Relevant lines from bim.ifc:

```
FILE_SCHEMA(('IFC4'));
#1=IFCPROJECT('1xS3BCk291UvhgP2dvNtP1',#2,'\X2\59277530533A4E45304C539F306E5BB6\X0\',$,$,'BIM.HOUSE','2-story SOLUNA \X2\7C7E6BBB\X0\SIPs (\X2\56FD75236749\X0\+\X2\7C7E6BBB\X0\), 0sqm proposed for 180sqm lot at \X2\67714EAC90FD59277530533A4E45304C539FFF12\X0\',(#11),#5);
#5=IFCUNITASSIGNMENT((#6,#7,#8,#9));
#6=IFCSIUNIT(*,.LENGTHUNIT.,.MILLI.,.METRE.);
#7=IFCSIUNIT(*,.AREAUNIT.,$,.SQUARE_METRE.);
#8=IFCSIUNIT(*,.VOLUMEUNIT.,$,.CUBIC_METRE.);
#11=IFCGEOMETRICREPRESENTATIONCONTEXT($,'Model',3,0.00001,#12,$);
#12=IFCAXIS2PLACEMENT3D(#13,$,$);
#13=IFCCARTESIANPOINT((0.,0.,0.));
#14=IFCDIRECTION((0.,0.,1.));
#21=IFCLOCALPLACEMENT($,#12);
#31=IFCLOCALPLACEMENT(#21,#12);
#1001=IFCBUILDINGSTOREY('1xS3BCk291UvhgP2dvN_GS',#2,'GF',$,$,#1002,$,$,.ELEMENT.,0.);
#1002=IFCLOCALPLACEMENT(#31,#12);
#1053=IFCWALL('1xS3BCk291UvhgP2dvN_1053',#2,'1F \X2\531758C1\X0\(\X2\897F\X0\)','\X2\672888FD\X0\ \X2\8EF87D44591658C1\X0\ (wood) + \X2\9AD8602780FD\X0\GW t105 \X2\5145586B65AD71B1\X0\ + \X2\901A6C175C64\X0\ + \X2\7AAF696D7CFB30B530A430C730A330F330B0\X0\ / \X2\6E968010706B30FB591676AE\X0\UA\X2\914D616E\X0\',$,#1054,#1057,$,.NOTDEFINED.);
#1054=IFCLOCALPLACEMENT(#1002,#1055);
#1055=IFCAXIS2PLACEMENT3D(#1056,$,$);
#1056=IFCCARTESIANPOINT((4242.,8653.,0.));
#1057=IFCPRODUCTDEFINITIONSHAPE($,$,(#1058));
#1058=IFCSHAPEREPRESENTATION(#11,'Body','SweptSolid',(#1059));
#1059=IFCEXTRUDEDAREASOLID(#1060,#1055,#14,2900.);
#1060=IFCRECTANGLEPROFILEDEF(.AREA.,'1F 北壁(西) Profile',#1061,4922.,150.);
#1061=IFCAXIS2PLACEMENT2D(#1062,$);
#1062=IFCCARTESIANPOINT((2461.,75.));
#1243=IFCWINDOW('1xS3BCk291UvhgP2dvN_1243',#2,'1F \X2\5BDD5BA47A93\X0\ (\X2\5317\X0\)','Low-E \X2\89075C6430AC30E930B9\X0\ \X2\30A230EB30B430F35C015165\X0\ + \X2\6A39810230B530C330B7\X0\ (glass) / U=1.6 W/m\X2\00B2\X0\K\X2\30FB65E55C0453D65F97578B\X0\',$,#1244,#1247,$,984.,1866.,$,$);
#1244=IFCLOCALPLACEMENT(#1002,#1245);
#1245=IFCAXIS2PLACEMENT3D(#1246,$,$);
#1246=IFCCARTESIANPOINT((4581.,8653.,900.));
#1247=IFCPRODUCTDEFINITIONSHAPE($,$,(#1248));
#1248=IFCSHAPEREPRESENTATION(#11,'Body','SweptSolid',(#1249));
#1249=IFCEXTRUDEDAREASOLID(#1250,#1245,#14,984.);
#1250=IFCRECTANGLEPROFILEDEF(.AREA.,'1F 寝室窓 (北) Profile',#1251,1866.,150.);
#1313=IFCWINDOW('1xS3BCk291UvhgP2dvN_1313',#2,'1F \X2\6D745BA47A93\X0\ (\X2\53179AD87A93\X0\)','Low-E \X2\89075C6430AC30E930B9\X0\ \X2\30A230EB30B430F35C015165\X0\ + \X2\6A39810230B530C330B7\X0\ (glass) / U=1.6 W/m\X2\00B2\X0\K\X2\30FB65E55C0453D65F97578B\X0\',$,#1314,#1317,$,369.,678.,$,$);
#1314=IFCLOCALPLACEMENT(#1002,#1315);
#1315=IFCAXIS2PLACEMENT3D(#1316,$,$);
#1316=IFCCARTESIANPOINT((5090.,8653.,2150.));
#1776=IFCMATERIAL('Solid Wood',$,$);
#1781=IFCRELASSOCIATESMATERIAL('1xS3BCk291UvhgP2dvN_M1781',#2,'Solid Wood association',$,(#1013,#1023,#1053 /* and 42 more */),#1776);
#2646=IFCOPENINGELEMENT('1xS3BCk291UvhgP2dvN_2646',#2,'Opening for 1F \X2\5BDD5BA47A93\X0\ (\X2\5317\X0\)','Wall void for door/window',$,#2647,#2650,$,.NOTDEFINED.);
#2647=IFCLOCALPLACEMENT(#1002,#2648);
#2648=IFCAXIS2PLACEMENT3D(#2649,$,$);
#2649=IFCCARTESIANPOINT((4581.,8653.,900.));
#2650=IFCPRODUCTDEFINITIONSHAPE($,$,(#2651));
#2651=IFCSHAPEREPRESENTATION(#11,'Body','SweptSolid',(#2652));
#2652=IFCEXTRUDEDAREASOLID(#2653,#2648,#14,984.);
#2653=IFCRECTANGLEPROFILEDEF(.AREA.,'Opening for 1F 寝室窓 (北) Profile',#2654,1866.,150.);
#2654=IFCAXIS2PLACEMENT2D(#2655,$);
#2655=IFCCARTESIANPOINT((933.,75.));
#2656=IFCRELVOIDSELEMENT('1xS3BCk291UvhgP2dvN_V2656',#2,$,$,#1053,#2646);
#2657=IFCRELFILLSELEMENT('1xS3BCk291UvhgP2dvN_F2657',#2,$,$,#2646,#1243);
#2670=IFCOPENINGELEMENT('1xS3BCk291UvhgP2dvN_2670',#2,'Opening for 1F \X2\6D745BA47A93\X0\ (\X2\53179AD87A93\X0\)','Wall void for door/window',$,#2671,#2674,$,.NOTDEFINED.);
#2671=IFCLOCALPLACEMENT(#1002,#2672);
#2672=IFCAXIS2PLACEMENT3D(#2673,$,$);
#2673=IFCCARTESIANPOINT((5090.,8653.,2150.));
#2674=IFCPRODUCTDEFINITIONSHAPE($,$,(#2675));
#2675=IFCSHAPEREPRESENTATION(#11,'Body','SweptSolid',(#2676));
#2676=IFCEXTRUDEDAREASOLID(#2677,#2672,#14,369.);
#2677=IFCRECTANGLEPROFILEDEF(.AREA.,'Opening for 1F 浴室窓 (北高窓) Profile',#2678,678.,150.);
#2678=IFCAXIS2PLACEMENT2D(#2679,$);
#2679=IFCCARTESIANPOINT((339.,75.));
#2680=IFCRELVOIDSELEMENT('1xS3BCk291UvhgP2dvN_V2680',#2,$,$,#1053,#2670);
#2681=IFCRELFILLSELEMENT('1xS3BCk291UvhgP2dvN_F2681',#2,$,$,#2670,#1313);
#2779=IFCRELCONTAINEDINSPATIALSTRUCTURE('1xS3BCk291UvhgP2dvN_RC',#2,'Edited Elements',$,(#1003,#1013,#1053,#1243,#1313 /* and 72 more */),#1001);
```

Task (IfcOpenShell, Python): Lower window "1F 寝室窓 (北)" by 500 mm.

```python
import numpy as np
import ifcopenshell
import ifcopenshell.api.geometry
import ifcopenshell.util.placement
import ifcopenshell.util.unit

model = ifcopenshell.open("bim.ifc")
unit_scale = ifcopenshell.util.unit.calculate_unit_scale(model)

window = model.by_guid("1xS3BCk291UvhgP2dvN_1243")
opening = window.FillsVoids[0].RelatingOpeningElement
dz = -0.5 / unit_scale

shift = np.array([0.0, 0.0, dz])
# The window is not placed relative to its opening, so move both.
for product in (opening, window):
    matrix = ifcopenshell.util.placement.get_local_placement(product.ObjectPlacement)
    matrix[:3, 3] += shift
    ifcopenshell.api.geometry.edit_object_placement(model, product=product, matrix=matrix, is_si=False)

print(f"moved by {dz * unit_scale:+.3f} m")

model.write("bim-out.ifc")
```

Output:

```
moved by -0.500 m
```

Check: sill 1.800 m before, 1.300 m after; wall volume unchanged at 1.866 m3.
